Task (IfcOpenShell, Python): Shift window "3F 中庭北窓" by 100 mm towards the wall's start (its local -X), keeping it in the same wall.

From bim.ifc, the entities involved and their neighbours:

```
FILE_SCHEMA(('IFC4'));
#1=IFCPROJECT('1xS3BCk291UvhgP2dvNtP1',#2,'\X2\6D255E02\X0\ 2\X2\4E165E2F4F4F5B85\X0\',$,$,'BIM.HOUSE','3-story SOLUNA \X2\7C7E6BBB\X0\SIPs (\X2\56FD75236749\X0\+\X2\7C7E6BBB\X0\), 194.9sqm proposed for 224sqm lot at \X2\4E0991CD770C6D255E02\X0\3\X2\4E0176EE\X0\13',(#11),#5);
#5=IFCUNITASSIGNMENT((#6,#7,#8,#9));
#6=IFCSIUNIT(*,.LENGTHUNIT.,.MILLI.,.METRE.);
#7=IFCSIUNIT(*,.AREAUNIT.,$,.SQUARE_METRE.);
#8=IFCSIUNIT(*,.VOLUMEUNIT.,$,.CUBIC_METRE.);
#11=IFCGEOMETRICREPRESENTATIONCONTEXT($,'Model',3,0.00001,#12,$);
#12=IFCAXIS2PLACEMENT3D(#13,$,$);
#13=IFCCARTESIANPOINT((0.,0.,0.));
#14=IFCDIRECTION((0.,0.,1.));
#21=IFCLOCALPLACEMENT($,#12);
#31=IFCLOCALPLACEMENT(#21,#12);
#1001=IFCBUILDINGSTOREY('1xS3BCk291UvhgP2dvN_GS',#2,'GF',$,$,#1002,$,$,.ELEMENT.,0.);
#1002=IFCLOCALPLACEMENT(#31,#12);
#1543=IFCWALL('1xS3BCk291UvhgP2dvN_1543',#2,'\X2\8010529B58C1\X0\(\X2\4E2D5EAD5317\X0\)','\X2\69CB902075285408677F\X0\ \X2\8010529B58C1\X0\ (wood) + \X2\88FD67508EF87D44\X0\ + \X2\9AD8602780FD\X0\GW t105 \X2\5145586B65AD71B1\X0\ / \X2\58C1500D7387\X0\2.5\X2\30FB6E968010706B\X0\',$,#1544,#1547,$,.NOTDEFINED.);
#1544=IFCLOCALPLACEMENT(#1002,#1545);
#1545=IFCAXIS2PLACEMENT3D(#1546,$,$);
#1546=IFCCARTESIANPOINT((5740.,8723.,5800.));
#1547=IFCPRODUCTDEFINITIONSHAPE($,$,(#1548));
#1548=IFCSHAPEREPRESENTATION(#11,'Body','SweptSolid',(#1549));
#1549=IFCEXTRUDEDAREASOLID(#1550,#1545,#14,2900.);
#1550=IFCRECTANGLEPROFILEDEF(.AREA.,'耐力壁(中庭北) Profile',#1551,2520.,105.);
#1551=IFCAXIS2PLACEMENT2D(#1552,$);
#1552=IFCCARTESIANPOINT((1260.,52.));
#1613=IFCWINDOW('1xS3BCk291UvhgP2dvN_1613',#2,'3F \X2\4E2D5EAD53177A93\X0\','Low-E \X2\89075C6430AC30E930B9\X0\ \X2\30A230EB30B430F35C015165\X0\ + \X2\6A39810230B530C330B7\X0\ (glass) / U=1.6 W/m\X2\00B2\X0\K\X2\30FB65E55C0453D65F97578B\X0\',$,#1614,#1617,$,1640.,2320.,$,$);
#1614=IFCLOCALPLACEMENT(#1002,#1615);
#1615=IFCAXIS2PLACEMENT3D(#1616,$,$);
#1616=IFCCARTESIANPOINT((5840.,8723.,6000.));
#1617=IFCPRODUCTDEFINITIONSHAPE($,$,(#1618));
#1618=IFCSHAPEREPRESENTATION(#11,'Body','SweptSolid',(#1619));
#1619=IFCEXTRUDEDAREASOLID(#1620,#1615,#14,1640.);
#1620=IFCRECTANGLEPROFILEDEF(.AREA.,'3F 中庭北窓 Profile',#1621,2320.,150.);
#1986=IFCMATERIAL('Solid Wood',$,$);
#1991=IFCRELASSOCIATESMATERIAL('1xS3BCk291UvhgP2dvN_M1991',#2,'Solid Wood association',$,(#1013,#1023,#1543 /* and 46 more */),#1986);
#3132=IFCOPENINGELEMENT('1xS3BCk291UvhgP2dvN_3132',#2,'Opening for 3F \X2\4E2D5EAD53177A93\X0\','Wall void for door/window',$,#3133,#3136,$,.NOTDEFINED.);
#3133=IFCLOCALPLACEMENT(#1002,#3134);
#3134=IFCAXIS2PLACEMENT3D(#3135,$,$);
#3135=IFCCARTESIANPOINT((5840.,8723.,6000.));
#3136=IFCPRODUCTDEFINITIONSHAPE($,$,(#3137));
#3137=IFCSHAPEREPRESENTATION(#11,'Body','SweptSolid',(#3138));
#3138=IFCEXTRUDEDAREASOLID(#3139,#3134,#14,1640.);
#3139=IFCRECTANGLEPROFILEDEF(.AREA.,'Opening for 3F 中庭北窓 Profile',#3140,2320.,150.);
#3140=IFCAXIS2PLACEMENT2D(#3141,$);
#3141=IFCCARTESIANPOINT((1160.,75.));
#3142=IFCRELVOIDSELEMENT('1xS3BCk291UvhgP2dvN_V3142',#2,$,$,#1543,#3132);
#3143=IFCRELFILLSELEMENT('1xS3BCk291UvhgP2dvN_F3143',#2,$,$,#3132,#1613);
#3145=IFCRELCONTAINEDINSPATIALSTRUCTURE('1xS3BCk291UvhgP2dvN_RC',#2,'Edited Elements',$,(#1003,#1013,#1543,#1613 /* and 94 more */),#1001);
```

```python
import ifcopenshell
import ifcopenshell.api.geometry
import ifcopenshell.util.placement
import ifcopenshell.util.unit

model = ifcopenshell.open("bim.ifc")
unit_scale = ifcopenshell.util.unit.calculate_unit_scale(model)

window = model.by_guid("1xS3BCk291UvhgP2dvN_1613")
opening = window.FillsVoids[0].RelatingOpeningElement
wall = opening.VoidsElements[0].RelatingBuildingElement

wall_matrix = ifcopenshell.util.placement.get_local_placement(wall.ObjectPlacement)
shift = wall_matrix[:3, 0] * -0.1 / unit_scale
before = ifcopenshell.util.placement.get_local_placement(window.ObjectPlacement)[:3, 3].copy()

# The window is not placed relative to its opening, so move both.
for product in (opening, window):
    matrix = ifcopenshell.util.placement.get_local_placement(product.ObjectPlacement)
    matrix[:3, 3] += shift
    ifcopenshell.api.geometry.edit_object_placement(model, product=product, matrix=matrix, is_si=False)

after = ifcopenshell.util.placement.get_local_placement(window.ObjectPlacement)[:3, 3]
print("window moved by", (after - before).round(3) + 0.0)

model.write("bim-out.ifc")
```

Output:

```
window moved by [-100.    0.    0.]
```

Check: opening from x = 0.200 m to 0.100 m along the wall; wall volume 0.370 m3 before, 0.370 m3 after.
